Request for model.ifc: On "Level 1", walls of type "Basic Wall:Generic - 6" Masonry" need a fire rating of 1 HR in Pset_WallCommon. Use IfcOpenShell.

First a look at what the model holds.

```python
import ifcopenshell
import ifcopenshell.util.element

model = ifcopenshell.open("model.ifc")
print(model.schema)
storey = next(s for s in model.by_type("IfcBuildingStorey") if s.Name == "Level 1")
walls = [e for e in ifcopenshell.util.element.get_decomposition(storey) if e.is_a("IfcWall")]
seen = {}
for e in walls:
    element_type = ifcopenshell.util.element.get_type(e)
    key = (element_type.Name if element_type != e and element_type else None, ifcopenshell.util.element.get_pset(e, "Pset_WallCommon", "FireRating"))
    seen[key] = seen.get(key, 0) + 1
for (name, value), count in sorted(seen.items(), key=str):
    print(count, "x", name, "|", value)
```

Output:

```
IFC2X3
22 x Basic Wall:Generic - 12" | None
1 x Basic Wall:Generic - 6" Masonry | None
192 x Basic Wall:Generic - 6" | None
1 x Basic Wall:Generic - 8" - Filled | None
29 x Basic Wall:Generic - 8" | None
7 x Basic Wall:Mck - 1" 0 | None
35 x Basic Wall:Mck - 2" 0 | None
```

```python
import ifcopenshell
import ifcopenshell.api.pset
import ifcopenshell.util.element

model = ifcopenshell.open("model.ifc")

storey = next(s for s in model.by_type("IfcBuildingStorey") if s.Name == "Level 1")
walls = [e for e in ifcopenshell.util.element.get_decomposition(storey) if e.is_a("IfcWall")]

count = 0
for e in walls:
    element_type = ifcopenshell.util.element.get_type(e)
    if element_type in (None, e) or element_type.Name != 'Basic Wall:Generic - 6" Masonry':
        continue
    # add_pset returns the element's existing set when there is one.
    pset = ifcopenshell.api.pset.add_pset(model, product=e, name="Pset_WallCommon")
    ifcopenshell.api.pset.edit_pset(model, pset=pset, properties={"FireRating": "1 HR"})
    count += 1

print(count, "walls updated")

model.write("model_edited.ifc")
```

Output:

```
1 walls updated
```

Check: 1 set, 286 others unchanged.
